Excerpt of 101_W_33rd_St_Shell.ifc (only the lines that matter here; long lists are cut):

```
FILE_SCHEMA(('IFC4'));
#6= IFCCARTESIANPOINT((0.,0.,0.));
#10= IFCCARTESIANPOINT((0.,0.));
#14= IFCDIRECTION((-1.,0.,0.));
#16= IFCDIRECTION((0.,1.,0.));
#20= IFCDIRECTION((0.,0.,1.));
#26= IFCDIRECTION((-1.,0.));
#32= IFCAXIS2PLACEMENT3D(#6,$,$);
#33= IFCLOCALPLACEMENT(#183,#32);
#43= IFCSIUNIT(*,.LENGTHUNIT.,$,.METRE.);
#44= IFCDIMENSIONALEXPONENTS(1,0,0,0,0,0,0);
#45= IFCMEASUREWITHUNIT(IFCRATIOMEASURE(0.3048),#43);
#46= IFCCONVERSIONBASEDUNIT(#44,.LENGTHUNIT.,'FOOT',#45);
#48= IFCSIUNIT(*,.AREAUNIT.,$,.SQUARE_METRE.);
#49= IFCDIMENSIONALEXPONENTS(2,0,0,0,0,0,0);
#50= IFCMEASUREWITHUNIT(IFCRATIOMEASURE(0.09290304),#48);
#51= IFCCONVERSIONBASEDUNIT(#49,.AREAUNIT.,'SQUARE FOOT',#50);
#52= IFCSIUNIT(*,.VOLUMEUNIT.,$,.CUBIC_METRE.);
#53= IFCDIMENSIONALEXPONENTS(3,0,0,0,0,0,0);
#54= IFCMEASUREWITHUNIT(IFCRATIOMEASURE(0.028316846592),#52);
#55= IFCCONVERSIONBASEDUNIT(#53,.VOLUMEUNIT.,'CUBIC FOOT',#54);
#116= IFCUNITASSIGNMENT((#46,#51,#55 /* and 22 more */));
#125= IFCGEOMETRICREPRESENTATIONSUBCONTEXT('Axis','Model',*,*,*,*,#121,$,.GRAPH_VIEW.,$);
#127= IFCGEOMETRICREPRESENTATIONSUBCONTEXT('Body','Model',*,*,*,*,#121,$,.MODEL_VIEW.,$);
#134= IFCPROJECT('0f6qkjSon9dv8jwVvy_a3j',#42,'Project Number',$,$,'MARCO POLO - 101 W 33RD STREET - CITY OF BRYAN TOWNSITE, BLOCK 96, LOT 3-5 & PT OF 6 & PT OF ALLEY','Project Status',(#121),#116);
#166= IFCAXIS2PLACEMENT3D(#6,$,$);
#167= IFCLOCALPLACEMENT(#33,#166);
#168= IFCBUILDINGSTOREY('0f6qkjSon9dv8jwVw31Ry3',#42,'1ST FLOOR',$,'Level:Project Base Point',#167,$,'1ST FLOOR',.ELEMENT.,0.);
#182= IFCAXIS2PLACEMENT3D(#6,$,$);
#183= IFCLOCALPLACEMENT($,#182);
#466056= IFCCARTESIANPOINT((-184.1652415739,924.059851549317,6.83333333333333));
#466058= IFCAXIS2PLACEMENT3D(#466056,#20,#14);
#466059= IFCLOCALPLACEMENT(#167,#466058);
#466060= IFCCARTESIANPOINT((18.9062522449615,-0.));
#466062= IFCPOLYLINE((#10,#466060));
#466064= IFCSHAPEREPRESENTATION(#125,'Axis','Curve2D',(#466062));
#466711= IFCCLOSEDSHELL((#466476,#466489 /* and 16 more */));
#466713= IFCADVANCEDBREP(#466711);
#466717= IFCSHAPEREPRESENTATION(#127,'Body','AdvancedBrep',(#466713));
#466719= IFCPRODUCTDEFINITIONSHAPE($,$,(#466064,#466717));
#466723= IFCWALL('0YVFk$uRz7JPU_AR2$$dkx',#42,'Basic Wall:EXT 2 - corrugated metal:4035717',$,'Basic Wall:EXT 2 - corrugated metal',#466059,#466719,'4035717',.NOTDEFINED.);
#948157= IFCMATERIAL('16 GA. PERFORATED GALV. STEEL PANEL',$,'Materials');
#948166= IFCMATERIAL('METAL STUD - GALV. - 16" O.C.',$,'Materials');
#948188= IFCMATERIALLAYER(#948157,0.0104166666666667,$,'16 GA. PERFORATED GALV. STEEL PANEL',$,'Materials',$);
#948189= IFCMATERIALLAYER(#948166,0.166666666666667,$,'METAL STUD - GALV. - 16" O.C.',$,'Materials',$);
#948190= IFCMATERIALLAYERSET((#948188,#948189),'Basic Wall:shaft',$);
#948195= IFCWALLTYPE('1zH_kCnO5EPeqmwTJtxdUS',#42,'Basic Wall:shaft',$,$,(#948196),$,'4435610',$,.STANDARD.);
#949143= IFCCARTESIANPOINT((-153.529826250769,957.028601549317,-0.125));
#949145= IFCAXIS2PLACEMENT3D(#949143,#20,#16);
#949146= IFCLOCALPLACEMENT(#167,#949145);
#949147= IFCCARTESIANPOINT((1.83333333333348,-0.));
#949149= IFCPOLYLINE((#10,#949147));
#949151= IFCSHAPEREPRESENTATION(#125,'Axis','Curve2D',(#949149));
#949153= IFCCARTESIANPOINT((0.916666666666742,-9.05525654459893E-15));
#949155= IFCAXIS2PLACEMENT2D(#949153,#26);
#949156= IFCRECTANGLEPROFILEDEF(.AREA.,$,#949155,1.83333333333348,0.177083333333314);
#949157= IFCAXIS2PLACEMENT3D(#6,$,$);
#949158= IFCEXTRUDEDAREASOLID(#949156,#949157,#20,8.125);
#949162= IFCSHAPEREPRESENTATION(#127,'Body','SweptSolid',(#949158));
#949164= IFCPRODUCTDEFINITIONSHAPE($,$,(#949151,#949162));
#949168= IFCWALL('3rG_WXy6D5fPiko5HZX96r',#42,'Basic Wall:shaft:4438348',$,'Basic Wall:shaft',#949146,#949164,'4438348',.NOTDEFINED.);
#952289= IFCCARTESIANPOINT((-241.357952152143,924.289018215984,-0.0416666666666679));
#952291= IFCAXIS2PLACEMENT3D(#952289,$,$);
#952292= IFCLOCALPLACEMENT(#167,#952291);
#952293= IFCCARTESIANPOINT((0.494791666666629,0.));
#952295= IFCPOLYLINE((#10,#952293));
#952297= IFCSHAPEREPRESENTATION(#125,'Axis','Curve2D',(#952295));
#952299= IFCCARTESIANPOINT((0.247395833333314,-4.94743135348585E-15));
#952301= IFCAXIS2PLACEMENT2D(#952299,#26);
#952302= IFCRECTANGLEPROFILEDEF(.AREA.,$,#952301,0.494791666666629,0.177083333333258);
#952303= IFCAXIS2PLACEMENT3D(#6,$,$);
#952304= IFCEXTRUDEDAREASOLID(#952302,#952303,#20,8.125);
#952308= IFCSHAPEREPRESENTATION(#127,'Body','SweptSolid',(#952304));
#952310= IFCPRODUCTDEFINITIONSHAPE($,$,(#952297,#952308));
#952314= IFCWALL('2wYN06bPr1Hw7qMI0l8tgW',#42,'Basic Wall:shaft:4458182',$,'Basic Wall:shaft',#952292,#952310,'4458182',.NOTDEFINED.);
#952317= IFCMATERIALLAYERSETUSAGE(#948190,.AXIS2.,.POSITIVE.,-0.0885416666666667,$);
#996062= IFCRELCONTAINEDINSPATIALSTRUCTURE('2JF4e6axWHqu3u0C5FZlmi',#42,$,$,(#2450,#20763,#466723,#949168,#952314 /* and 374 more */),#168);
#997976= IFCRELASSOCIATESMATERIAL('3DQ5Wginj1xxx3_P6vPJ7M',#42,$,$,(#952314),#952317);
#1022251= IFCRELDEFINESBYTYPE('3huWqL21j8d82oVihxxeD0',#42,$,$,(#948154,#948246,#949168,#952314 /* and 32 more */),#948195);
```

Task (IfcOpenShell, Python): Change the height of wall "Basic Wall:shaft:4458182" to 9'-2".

```python
import ifcopenshell
import ifcopenshell.geom
import ifcopenshell.util.representation
import ifcopenshell.util.shape
import ifcopenshell.util.unit

model = ifcopenshell.open("101_W_33rd_St_Shell.ifc")
unit_scale = ifcopenshell.util.unit.calculate_unit_scale(model)
settings = ifcopenshell.geom.settings()


def volume(element):
    """Net volume in cubic metres, openings subtracted."""
    shape = ifcopenshell.geom.create_shape(settings, element)
    return ifcopenshell.util.shape.get_volume(shape.geometry)


wall = model.by_guid("2wYN06bPr1Hw7qMI0l8tgW")
before = volume(wall)

body = ifcopenshell.util.representation.get_representation(wall, "Model", "Body")
solid = body.Items[0]
old_height = solid.Depth
solid.Depth = 110 * 0.0254 / unit_scale
after = volume(wall)

print(f"height {old_height:g} -> {solid.Depth:g}, volume {before:.3f} -> {after:.3f} m3")

model.write("101_W_33rd_St_Shell_updated.ifc")
```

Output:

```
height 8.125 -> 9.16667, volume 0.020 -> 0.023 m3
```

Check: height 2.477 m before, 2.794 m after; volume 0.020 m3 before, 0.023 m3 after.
